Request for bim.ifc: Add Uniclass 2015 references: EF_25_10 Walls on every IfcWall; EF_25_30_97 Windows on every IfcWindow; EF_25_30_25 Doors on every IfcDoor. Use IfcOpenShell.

First a look at what the model holds.

```python
import ifcopenshell

model = ifcopenshell.open("bim.ifc")
print(model.schema)
print("classifications:", [c.Name for c in model.by_type("IfcClassification")])
for ifc_class in ("IfcDoor", "IfcRoof", "IfcStair", "IfcWall", "IfcWindow"):
    print(ifc_class, len(model.by_type(ifc_class)))
```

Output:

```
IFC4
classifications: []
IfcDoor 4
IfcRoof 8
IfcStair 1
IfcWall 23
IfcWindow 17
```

```python
import ifcopenshell
import ifcopenshell.api.classification

model = ifcopenshell.open("bim.ifc")

system = ifcopenshell.api.classification.add_classification(model, classification="Uniclass 2015")

codes = {
    "IfcWall": ("EF_25_10", "Walls"),
    "IfcWindow": ("EF_25_30_97", "Windows"),
    "IfcDoor": ("EF_25_30_25", "Doors"),
}
for ifc_class, (code, name) in codes.items():
    products = model.by_type(ifc_class)
    ifcopenshell.api.classification.add_reference(
        model, products=products, classification=system, identification=code, name=name
    )
    print(code, len(products))

model.write("bim_v2.ifc")
```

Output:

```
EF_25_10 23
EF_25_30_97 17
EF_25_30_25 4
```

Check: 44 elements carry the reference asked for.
